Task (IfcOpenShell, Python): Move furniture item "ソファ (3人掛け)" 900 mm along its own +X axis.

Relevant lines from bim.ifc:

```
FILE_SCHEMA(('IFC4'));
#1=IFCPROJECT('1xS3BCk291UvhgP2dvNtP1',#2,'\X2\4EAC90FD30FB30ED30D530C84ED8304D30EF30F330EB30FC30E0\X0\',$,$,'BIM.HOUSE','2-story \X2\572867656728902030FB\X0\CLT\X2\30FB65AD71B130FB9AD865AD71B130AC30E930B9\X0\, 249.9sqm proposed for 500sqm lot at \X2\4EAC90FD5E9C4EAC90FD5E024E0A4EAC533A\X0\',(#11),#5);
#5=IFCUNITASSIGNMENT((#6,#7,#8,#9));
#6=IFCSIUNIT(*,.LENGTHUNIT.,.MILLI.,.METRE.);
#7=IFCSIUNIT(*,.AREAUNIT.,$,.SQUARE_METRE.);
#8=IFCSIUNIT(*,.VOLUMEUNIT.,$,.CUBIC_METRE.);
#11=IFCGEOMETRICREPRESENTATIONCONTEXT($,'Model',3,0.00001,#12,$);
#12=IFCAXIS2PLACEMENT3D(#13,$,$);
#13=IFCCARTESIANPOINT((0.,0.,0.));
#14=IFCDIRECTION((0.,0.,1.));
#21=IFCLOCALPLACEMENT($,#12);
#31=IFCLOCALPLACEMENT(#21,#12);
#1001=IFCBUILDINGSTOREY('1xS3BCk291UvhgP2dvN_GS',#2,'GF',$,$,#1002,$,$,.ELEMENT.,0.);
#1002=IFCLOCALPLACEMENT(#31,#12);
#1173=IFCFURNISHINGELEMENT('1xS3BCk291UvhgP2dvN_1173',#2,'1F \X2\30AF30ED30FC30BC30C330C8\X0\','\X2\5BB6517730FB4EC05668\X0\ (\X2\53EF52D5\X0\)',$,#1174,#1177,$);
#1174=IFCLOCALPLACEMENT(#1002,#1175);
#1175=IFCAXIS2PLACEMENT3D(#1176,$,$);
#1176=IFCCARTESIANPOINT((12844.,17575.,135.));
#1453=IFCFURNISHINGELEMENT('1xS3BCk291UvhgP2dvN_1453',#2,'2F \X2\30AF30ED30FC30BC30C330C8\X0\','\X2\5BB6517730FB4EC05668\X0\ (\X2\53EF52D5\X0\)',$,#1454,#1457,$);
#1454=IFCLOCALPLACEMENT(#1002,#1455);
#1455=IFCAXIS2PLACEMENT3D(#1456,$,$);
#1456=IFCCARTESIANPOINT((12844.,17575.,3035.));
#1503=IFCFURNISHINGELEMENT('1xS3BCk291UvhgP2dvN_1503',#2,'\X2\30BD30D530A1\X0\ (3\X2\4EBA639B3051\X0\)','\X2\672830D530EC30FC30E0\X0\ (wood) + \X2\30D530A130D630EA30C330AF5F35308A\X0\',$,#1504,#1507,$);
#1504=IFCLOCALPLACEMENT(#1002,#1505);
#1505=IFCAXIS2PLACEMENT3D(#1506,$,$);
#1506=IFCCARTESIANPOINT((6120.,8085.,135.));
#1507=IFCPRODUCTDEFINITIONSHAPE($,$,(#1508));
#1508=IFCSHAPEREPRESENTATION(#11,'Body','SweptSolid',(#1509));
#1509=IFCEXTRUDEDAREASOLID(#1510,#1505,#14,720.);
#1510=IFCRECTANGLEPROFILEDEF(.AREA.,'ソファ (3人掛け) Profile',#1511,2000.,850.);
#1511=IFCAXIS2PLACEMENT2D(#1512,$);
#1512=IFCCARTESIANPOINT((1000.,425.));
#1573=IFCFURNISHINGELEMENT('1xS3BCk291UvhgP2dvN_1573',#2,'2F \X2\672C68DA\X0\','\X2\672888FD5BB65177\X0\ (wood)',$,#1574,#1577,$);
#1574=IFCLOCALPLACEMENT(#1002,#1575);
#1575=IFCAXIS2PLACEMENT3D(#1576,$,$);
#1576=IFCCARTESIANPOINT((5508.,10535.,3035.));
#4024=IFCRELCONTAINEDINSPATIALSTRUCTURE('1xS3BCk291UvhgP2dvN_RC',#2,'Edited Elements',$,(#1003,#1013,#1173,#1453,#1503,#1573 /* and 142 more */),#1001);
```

```python
import ifcopenshell
import ifcopenshell.api.geometry
import ifcopenshell.util.placement

model = ifcopenshell.open("bim.ifc")

item = model.by_guid("1xS3BCk291UvhgP2dvN_1503")
matrix = ifcopenshell.util.placement.get_local_placement(item.ObjectPlacement)
matrix[:3, 3] += matrix[:3, 0] * 900.0
ifcopenshell.api.geometry.edit_object_placement(model, product=item, matrix=matrix, is_si=False)

print(ifcopenshell.util.placement.get_local_placement(item.ObjectPlacement).round(3) + 0.0)

model.write("bim_rev.ifc")
```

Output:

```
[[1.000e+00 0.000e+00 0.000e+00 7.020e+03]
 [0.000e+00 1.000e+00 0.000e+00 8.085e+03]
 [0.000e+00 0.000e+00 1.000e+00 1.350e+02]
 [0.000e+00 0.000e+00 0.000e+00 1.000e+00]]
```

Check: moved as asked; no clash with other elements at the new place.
